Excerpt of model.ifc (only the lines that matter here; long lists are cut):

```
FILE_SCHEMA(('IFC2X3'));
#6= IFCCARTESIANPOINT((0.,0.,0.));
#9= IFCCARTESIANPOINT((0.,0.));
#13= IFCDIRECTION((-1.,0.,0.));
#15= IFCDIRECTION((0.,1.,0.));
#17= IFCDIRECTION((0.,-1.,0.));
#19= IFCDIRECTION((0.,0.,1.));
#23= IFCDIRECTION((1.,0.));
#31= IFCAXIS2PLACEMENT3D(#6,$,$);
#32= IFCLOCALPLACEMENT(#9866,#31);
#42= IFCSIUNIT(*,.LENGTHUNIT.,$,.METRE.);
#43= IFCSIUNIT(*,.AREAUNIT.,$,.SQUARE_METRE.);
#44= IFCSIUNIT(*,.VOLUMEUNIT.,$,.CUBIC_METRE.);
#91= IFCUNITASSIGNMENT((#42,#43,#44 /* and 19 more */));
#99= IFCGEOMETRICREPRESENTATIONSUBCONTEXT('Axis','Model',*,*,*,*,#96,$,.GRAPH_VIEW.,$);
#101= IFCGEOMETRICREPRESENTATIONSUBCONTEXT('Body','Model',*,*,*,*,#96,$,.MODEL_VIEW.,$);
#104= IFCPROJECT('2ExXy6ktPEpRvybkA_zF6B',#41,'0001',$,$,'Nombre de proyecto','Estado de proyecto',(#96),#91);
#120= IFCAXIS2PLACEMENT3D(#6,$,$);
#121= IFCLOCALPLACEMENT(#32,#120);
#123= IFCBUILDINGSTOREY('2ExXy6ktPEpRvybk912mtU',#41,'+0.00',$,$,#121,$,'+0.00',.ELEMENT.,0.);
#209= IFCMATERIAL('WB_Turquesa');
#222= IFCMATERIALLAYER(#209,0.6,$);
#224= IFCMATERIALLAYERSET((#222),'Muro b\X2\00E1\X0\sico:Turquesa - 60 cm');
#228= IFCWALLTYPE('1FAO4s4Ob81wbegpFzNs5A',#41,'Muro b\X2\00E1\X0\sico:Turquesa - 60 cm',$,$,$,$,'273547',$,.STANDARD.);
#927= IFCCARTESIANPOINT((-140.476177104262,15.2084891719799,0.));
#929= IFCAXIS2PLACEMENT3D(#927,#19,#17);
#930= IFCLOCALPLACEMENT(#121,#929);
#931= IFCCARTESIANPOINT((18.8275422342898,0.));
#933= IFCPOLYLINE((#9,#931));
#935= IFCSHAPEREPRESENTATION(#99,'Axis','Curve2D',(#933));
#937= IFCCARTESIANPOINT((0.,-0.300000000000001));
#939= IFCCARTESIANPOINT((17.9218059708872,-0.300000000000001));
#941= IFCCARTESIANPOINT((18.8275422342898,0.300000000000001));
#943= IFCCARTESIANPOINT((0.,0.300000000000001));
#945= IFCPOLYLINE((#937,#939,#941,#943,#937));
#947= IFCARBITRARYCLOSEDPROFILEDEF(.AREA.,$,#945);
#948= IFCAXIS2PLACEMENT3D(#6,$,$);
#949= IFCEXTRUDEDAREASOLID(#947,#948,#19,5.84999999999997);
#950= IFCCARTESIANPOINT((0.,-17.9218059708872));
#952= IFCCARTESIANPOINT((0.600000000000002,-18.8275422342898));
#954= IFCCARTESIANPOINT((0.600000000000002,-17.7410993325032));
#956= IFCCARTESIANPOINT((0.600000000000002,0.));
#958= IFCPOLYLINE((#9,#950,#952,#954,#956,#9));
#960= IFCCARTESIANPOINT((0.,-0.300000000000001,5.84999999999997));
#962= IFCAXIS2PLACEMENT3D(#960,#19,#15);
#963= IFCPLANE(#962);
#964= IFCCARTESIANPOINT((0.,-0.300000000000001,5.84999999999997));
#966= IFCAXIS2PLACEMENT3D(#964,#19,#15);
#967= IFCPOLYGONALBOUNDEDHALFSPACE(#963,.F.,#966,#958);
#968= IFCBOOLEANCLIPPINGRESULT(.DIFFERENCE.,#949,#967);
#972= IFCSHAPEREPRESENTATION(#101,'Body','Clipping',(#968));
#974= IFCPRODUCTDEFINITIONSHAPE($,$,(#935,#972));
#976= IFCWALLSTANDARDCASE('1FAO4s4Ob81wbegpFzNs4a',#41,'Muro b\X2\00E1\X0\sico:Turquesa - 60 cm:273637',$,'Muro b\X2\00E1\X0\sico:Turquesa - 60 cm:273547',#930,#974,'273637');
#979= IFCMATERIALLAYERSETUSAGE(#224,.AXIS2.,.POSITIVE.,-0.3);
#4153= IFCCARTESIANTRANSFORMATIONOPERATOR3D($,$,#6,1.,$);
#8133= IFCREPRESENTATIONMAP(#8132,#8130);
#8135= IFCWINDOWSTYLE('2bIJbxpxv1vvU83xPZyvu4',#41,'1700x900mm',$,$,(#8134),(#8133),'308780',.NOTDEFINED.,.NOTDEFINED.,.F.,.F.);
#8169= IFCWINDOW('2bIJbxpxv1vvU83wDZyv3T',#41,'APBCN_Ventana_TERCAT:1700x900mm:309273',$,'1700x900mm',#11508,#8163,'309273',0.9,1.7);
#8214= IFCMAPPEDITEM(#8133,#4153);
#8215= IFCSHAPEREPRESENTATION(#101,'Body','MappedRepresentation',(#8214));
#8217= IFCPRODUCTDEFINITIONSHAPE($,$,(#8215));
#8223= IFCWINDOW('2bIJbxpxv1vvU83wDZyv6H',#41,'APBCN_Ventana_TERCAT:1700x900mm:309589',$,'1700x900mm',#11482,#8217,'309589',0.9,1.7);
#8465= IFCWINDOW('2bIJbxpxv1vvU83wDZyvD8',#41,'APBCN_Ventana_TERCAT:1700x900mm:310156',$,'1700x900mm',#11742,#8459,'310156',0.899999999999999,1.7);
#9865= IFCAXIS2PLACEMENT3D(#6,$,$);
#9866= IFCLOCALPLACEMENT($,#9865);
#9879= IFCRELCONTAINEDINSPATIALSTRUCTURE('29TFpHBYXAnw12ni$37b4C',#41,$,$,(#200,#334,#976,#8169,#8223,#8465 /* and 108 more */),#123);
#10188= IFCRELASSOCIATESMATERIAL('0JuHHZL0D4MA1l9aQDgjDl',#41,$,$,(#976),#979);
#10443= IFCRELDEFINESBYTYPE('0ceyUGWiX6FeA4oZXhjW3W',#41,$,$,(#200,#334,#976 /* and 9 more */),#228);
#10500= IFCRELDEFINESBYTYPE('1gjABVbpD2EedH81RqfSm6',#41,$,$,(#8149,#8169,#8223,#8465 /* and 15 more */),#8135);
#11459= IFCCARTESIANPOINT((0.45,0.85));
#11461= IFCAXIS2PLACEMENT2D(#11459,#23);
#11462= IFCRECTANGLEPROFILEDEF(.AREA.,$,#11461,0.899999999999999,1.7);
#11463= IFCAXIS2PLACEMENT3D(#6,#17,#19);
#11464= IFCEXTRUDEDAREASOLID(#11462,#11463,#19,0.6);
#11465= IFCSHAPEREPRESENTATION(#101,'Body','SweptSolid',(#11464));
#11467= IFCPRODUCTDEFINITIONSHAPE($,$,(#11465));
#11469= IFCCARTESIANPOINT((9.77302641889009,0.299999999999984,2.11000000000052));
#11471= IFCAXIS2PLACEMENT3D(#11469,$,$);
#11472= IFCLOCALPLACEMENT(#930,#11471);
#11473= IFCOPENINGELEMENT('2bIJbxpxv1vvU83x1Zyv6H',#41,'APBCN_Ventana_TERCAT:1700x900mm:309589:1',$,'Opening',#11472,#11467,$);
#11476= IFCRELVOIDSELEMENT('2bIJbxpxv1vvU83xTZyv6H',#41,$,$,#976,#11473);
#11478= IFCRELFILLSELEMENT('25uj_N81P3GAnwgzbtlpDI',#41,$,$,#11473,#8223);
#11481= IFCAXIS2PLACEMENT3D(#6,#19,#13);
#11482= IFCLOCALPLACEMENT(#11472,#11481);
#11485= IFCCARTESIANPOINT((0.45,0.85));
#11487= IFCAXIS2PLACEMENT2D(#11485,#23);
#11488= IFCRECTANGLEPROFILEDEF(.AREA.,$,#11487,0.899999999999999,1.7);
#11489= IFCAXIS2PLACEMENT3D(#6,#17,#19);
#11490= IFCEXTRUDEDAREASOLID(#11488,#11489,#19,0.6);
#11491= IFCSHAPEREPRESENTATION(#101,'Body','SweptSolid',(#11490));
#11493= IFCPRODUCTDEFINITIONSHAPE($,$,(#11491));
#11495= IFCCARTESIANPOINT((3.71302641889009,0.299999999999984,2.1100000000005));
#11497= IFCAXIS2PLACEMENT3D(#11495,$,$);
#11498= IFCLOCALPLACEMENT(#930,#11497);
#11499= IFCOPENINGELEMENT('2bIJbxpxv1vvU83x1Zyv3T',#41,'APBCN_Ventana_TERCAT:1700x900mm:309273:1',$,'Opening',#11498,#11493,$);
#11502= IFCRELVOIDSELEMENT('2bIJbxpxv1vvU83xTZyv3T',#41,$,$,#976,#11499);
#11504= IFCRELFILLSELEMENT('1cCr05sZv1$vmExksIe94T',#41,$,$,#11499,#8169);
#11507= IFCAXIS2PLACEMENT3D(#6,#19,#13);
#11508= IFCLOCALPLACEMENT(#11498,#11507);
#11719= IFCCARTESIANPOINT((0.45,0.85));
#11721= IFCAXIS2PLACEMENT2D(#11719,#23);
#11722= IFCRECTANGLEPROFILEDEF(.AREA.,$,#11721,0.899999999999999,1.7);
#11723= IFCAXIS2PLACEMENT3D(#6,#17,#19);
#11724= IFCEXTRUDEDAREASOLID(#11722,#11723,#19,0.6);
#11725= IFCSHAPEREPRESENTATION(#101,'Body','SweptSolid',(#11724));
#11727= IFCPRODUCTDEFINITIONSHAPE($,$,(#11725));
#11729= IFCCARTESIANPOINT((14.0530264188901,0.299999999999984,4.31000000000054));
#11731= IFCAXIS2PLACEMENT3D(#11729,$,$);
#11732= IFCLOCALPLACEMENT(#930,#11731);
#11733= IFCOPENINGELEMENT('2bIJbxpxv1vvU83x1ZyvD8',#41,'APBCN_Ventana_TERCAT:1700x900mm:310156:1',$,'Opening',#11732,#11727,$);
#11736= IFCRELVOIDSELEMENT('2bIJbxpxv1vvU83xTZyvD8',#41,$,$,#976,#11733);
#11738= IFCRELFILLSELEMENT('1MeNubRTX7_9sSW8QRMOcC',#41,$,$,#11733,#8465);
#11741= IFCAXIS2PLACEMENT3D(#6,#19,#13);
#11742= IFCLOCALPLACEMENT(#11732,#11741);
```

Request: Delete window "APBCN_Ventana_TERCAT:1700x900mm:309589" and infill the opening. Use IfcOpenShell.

```python
import ifcopenshell
import ifcopenshell.api.feature
import ifcopenshell.api.root
import ifcopenshell.geom
import ifcopenshell.util.shape

model = ifcopenshell.open("model.ifc")
settings = ifcopenshell.geom.settings()


def volume(element):
    """Net volume in cubic metres, openings subtracted."""
    shape = ifcopenshell.geom.create_shape(settings, element)
    return ifcopenshell.util.shape.get_volume(shape.geometry)


window = model.by_id(8223)
opening = window.FillsVoids[0].RelatingOpeningElement
wall = opening.VoidsElements[0].RelatingBuildingElement
before = volume(wall)

ifcopenshell.api.root.remove_product(model, product=window)
ifcopenshell.api.feature.remove_feature(model, feature=opening)

after = volume(wall)

print(f"wall volume {before:.3f} -> {after:.3f} m3")

model.write("model_v2.ifc")
```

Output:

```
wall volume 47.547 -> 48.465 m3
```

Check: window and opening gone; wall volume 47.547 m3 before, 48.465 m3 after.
